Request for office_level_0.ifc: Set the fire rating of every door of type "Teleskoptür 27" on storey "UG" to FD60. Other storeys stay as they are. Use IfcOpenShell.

First a look at what the model holds.

```python
import ifcopenshell
import ifcopenshell.util.element

model = ifcopenshell.open("office_level_0.ifc")
print(model.schema)
storey = next(s for s in model.by_type("IfcBuildingStorey") if s.Name == "UG")
doors = [e for e in ifcopenshell.util.element.get_decomposition(storey) if e.is_a("IfcDoor")]
seen = {}
for e in doors:
    element_type = ifcopenshell.util.element.get_type(e)
    key = (element_type.Name if element_type != e and element_type else None, ifcopenshell.util.element.get_pset(e, "Pset_DoorCommon", "FireRating"))
    seen[key] = seen.get(key, 0) + 1
for (name, value), count in sorted(seen.items(), key=str):
    print(count, "x", name, "|", value)
```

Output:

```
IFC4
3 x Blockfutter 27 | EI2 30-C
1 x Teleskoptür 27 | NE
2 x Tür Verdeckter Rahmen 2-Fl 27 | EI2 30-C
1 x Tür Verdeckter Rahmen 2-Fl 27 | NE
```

```python
import ifcopenshell
import ifcopenshell.api.pset
import ifcopenshell.util.element

model = ifcopenshell.open("office_level_0.ifc")

storey = next(s for s in model.by_type("IfcBuildingStorey") if s.Name == "UG")
doors = [e for e in ifcopenshell.util.element.get_decomposition(storey) if e.is_a("IfcDoor")]

count = 0
for e in doors:
    element_type = ifcopenshell.util.element.get_type(e)
    if element_type in (None, e) or element_type.Name != "Teleskoptür 27":
        continue
    # add_pset returns the element's existing set when there is one.
    pset = ifcopenshell.api.pset.add_pset(model, product=e, name="Pset_DoorCommon")
    ifcopenshell.api.pset.edit_pset(model, pset=pset, properties={"FireRating": "FD60"})
    count += 1

print(count, "doors updated")

model.write("office_level_0_rev.ifc")
```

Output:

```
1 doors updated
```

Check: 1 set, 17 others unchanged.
